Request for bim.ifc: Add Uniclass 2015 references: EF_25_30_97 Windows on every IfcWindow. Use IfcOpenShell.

First a look at what the model holds.

```python
import ifcopenshell

model = ifcopenshell.open("bim.ifc")
print(model.schema)
print("classifications:", [c.Name for c in model.by_type("IfcClassification")])
for ifc_class in ("IfcDoor", "IfcRoof", "IfcStair", "IfcWall", "IfcWindow"):
    print(ifc_class, len(model.by_type(ifc_class)))
```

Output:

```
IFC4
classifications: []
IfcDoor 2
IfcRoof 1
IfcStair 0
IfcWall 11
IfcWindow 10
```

```python
import ifcopenshell
import ifcopenshell.api.classification

model = ifcopenshell.open("bim.ifc")

system = ifcopenshell.api.classification.add_classification(model, classification="Uniclass 2015")

codes = {
    "IfcWindow": ("EF_25_30_97", "Windows"),
}
for ifc_class, (code, name) in codes.items():
    products = model.by_type(ifc_class)
    ifcopenshell.api.classification.add_reference(
        model, products=products, classification=system, identification=code, name=name
    )
    print(code, len(products))

model.write("bim_updated.ifc")
```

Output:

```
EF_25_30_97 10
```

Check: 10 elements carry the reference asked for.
